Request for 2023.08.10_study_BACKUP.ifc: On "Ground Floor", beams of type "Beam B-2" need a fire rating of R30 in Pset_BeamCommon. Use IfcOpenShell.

First a look at what the model holds.

```python
import ifcopenshell
import ifcopenshell.util.element

model = ifcopenshell.open("2023.08.10_study_BACKUP.ifc")
print(model.schema)
storey = next(s for s in model.by_type("IfcBuildingStorey") if s.Name == "Ground Floor")
beams = [e for e in ifcopenshell.util.element.get_decomposition(storey) if e.is_a("IfcBeam")]
seen = {}
for e in beams:
    element_type = ifcopenshell.util.element.get_type(e)
    key = (element_type.Name if element_type != e and element_type else None, ifcopenshell.util.element.get_pset(e, "Pset_BeamCommon", "FireRating"))
    seen[key] = seen.get(key, 0) + 1
for (name, value), count in sorted(seen.items(), key=str):
    print(count, "x", name, "|", value)
```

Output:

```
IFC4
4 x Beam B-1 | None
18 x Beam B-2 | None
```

```python
import ifcopenshell
import ifcopenshell.api.pset
import ifcopenshell.util.element

model = ifcopenshell.open("2023.08.10_study_BACKUP.ifc")

storey = next(s for s in model.by_type("IfcBuildingStorey") if s.Name == "Ground Floor")
beams = [e for e in ifcopenshell.util.element.get_decomposition(storey) if e.is_a("IfcBeam")]

count = 0
for e in beams:
    element_type = ifcopenshell.util.element.get_type(e)
    if element_type in (None, e) or element_type.Name != "Beam B-2":
        continue
    # add_pset returns the element's existing set when there is one.
    pset = ifcopenshell.api.pset.add_pset(model, product=e, name="Pset_BeamCommon")
    ifcopenshell.api.pset.edit_pset(model, pset=pset, properties={"FireRating": "R30"})
    count += 1

print(count, "beams updated")

model.write("2023.08.10_study_BACKUP_rev.ifc")
```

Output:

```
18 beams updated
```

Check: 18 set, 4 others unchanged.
